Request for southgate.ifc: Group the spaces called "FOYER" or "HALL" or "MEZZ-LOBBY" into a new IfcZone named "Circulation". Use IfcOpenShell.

First a look at what the model holds.

```python
import ifcopenshell

model = ifcopenshell.open("southgate.ifc")
print(model.schema)
seen = {}
for space in model.by_type("IfcSpace"):
    seen[space.LongName] = seen.get(space.LongName, 0) + 1
for name, count in sorted(seen.items(), key=str):
    print(count, "x", name)
print("zones:", [z.Name for z in model.by_type("IfcZone")][:20])
```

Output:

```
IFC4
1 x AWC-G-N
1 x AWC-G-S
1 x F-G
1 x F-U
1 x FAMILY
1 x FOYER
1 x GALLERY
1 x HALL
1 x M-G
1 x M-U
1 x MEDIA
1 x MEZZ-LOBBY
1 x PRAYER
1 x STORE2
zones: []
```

```python
import ifcopenshell
import ifcopenshell.api.group
import ifcopenshell.api.root

model = ifcopenshell.open("southgate.ifc")

names = {"FOYER", "HALL", "MEZZ-LOBBY"}
spaces = [s for s in model.by_type("IfcSpace") if s.LongName in names]

zone = ifcopenshell.api.root.create_entity(model, ifc_class="IfcZone", name="Circulation")
ifcopenshell.api.group.assign_group(model, products=spaces, group=zone)
print(len(spaces), "spaces in", zone.Name)

model.write("southgate_updated.ifc")
```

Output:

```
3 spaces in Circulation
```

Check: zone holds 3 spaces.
